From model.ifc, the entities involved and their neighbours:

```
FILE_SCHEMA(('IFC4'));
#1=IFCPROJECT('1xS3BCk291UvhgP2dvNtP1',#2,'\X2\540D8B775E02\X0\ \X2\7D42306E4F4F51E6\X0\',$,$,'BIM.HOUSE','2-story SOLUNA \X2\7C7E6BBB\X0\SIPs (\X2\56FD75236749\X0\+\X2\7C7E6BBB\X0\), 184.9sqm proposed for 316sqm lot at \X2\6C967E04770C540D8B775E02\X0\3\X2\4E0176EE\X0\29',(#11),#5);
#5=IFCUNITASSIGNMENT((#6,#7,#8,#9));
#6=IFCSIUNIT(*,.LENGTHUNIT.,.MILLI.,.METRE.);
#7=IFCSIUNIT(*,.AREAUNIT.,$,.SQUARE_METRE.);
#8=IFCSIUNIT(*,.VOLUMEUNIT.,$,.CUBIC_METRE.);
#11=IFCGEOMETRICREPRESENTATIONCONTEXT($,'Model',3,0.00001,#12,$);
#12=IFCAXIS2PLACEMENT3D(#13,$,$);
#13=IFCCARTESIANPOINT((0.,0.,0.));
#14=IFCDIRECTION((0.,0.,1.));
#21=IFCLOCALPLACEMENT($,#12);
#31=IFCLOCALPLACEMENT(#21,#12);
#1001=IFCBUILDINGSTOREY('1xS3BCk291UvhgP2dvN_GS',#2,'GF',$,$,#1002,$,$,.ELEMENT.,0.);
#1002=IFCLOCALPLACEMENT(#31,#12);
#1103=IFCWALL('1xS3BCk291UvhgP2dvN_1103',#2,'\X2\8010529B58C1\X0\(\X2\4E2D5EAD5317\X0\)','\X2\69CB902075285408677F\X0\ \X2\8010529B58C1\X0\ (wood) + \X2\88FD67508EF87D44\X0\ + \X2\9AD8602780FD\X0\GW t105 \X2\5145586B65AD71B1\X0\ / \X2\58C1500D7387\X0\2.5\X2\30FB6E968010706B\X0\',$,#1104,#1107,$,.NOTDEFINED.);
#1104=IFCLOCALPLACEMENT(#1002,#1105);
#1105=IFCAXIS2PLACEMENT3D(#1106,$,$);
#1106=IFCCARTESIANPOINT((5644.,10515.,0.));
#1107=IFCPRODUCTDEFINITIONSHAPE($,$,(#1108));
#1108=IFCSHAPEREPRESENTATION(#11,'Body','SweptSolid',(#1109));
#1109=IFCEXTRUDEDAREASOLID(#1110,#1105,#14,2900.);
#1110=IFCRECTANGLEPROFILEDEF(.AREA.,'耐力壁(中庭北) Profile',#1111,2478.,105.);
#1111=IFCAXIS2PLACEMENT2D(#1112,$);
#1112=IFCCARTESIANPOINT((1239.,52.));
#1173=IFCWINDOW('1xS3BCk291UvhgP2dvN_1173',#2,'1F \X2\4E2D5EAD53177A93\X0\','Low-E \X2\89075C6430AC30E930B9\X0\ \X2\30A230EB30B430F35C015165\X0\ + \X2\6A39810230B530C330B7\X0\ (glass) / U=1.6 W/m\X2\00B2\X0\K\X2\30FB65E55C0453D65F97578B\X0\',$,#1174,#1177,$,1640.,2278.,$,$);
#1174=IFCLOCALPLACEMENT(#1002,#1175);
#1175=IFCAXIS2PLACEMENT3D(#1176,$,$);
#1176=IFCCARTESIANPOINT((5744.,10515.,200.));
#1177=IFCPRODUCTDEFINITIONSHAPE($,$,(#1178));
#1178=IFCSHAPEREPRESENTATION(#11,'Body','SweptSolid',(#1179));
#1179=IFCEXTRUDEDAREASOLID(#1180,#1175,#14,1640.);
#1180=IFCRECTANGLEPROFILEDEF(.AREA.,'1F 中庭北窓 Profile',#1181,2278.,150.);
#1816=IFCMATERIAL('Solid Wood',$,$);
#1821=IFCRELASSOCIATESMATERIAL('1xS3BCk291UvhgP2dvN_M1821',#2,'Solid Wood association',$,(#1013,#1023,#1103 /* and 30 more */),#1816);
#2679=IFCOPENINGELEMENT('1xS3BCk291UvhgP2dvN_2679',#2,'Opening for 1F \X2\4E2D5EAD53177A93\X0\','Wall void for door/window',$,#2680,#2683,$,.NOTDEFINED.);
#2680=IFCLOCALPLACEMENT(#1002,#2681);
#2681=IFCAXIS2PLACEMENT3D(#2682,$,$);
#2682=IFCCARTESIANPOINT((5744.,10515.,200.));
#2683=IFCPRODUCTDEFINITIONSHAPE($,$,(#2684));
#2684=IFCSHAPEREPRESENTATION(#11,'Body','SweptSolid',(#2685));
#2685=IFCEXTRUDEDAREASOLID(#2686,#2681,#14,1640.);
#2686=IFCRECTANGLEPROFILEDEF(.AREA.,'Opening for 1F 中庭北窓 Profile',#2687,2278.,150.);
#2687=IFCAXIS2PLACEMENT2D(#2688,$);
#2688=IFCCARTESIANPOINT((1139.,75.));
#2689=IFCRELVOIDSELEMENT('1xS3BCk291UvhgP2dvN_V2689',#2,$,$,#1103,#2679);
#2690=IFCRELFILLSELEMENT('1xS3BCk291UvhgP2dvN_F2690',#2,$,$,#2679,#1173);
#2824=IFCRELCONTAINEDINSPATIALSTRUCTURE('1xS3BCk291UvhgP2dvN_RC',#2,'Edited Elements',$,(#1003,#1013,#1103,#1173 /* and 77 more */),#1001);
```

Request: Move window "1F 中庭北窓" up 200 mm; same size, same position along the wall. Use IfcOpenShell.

```python
import numpy as np
import ifcopenshell
import ifcopenshell.api.geometry
import ifcopenshell.util.placement
import ifcopenshell.util.unit

model = ifcopenshell.open("model.ifc")
unit_scale = ifcopenshell.util.unit.calculate_unit_scale(model)

window = model.by_id(1173)
opening = window.FillsVoids[0].RelatingOpeningElement
dz = 0.2 / unit_scale

shift = np.array([0.0, 0.0, dz])
# The window is not placed relative to its opening, so move both.
for product in (opening, window):
    matrix = ifcopenshell.util.placement.get_local_placement(product.ObjectPlacement)
    matrix[:3, 3] += shift
    ifcopenshell.api.geometry.edit_object_placement(model, product=product, matrix=matrix, is_si=False)

print(f"moved by {dz * unit_scale:+.3f} m")

model.write("model_updated.ifc")
```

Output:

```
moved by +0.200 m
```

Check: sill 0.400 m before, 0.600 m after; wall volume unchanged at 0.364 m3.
